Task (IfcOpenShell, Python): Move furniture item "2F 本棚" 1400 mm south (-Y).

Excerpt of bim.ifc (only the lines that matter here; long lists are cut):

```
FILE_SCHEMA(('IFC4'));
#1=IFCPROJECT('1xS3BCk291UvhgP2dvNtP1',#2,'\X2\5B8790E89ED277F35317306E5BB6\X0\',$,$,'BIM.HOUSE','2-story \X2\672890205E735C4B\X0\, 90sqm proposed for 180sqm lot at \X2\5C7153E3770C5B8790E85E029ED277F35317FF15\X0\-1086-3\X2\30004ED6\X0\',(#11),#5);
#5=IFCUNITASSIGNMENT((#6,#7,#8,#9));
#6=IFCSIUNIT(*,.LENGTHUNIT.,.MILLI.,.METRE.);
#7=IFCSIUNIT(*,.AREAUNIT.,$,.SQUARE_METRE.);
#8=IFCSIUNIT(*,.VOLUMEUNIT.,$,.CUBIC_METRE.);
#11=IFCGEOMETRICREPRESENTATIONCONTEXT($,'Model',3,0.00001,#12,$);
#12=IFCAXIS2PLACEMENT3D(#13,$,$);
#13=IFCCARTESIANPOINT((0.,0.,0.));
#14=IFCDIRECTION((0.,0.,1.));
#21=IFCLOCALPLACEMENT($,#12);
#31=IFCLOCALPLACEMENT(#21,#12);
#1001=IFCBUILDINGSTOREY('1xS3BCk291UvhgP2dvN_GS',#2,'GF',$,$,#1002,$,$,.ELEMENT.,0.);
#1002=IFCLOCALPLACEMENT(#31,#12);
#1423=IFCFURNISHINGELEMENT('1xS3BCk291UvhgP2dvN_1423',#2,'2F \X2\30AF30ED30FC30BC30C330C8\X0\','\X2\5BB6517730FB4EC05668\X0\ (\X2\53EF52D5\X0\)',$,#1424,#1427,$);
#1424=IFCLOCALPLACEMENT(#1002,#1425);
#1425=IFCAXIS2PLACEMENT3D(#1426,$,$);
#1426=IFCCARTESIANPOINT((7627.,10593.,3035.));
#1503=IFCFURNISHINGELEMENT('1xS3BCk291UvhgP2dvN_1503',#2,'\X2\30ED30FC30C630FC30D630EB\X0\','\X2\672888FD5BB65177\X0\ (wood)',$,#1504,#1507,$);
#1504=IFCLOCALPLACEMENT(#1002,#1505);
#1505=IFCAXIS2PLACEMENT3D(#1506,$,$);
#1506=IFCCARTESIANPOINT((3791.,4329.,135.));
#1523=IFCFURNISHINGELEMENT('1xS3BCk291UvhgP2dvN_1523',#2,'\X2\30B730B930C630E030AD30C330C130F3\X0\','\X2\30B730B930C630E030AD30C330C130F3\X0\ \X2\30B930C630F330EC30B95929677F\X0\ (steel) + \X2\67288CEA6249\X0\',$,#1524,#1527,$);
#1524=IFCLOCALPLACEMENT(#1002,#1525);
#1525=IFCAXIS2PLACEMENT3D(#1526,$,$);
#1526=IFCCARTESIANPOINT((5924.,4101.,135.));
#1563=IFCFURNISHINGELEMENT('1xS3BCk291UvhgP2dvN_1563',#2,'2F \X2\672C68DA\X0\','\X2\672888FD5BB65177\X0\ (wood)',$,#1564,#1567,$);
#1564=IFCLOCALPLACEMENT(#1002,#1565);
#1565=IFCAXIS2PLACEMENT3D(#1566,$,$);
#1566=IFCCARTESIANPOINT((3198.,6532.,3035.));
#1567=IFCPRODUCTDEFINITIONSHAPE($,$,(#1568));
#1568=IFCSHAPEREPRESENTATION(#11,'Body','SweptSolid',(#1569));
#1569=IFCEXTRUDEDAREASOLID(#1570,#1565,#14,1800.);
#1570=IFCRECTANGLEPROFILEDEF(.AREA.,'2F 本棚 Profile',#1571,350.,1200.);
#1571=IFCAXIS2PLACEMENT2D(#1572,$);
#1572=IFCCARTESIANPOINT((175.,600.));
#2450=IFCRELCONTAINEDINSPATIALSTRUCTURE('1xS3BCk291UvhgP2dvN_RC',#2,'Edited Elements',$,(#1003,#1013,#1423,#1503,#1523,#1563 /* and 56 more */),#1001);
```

```python
import ifcopenshell
import ifcopenshell.api.geometry
import ifcopenshell.util.placement
import ifcopenshell.util.unit

model = ifcopenshell.open("bim.ifc")
unit_scale = ifcopenshell.util.unit.calculate_unit_scale(model)

item = model.by_guid("1xS3BCk291UvhgP2dvN_1563")
matrix = ifcopenshell.util.placement.get_local_placement(item.ObjectPlacement)
matrix[1, 3] -= 1.4 / unit_scale
ifcopenshell.api.geometry.edit_object_placement(model, product=item, matrix=matrix, is_si=False)

print(ifcopenshell.util.placement.get_local_placement(item.ObjectPlacement).round(3) + 0.0)

model.write("bim_updated.ifc")
```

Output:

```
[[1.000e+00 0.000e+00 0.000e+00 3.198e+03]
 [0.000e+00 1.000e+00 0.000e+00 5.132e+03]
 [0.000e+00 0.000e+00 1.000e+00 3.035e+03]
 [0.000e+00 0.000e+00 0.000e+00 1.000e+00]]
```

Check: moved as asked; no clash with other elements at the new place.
